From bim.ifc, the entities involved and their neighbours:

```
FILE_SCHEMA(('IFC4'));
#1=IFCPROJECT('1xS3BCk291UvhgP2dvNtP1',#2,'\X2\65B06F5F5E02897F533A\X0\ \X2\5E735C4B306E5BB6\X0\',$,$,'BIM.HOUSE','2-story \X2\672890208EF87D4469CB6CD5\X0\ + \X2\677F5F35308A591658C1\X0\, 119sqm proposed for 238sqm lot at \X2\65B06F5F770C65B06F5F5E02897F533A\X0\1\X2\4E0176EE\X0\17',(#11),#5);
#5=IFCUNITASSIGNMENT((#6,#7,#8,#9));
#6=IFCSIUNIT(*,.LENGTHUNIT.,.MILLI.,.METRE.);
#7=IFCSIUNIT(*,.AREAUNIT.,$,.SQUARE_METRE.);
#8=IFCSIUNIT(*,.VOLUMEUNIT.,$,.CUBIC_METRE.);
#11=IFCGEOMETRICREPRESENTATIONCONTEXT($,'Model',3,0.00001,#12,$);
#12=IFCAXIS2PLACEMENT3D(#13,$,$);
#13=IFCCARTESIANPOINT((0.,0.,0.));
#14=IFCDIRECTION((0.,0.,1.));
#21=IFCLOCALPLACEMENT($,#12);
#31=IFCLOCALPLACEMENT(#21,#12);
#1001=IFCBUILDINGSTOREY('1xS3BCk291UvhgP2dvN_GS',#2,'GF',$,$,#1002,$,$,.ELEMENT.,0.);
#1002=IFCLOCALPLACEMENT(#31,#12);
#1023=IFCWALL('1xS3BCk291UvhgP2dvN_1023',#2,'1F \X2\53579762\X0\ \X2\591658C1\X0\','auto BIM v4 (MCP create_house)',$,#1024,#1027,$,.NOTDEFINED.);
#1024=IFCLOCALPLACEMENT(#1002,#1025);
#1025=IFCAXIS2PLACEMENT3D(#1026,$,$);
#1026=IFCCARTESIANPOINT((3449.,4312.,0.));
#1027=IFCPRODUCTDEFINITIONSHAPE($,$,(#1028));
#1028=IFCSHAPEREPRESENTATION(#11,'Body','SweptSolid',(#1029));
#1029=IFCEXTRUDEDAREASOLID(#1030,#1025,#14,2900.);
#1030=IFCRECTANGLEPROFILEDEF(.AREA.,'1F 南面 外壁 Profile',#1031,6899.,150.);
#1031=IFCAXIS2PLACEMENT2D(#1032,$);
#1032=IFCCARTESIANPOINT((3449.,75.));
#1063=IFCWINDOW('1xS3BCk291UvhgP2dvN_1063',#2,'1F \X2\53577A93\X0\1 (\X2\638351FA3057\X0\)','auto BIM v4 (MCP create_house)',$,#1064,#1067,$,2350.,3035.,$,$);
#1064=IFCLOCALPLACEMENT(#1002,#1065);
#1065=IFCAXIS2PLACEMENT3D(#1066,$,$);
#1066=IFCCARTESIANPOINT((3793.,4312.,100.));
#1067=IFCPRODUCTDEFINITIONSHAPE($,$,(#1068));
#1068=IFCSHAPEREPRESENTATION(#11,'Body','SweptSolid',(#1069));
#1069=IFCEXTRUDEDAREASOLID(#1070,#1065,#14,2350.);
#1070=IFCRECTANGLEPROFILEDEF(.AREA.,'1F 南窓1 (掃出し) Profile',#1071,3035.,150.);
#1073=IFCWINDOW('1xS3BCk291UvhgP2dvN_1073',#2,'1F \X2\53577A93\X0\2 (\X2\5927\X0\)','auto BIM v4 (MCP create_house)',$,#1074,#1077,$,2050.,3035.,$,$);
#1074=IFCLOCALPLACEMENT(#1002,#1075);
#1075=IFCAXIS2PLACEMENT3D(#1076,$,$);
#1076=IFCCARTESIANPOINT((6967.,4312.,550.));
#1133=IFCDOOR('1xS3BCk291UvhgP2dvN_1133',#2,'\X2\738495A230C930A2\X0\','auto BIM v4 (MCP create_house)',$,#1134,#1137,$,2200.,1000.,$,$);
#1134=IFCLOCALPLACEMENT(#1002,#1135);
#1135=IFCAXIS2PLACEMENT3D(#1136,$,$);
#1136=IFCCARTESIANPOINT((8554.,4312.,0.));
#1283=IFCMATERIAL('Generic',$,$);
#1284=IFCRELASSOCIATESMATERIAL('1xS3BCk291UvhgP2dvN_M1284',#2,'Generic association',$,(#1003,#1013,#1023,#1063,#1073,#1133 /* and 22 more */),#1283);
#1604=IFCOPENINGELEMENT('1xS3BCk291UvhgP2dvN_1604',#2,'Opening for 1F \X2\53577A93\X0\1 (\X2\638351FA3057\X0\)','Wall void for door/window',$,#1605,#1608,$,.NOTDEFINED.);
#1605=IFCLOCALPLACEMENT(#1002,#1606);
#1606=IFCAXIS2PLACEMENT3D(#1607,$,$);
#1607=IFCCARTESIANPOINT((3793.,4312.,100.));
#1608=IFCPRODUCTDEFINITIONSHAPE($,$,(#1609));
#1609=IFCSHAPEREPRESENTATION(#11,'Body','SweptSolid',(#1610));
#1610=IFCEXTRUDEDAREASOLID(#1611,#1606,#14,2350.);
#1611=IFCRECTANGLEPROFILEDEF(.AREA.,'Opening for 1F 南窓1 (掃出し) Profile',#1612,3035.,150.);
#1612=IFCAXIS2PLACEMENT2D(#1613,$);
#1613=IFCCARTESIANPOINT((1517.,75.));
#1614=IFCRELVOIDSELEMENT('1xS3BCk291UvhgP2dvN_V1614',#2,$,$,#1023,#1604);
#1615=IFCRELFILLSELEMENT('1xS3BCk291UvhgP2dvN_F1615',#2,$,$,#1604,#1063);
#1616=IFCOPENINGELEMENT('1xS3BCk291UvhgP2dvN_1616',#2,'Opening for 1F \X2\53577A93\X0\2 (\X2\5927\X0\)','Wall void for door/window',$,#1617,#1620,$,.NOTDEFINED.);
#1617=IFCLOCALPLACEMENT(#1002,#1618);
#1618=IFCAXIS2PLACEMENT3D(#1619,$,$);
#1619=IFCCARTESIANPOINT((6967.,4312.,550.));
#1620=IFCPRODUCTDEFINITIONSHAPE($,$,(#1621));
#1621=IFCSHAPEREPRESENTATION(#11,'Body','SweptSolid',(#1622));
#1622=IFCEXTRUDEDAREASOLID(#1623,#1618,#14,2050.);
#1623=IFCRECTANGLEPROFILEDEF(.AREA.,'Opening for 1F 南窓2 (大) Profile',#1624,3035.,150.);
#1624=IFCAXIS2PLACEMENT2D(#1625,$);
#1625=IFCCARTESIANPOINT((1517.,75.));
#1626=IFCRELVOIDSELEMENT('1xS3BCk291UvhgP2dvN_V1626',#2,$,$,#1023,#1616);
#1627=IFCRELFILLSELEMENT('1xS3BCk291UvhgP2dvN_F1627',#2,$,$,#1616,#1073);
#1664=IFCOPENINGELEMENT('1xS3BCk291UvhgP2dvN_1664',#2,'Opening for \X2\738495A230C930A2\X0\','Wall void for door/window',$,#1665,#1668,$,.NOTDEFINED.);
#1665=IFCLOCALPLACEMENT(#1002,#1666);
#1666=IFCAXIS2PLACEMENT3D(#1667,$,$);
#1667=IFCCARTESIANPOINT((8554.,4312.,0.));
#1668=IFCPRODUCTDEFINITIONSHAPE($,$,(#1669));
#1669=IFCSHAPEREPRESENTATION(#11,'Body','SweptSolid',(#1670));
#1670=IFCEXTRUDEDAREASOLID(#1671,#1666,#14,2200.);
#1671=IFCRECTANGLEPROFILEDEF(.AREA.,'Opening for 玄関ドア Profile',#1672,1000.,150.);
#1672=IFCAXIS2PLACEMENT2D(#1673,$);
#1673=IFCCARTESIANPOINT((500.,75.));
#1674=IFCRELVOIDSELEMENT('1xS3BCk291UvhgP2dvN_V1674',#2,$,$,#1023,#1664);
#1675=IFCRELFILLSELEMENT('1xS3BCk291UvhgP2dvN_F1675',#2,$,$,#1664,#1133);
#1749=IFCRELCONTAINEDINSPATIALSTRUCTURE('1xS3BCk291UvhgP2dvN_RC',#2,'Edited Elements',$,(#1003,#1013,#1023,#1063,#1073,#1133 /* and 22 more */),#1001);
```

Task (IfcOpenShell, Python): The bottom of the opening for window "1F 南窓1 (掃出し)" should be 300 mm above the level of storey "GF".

```python
import numpy as np
import ifcopenshell
import ifcopenshell.api.geometry
import ifcopenshell.geom
import ifcopenshell.util.element
import ifcopenshell.util.placement
import ifcopenshell.util.shape
import ifcopenshell.util.unit

model = ifcopenshell.open("bim.ifc")
unit_scale = ifcopenshell.util.unit.calculate_unit_scale(model)

window = model.by_id(1063)
opening = window.FillsVoids[0].RelatingOpeningElement
storey = ifcopenshell.util.element.get_container(window, ifc_class="IfcBuildingStorey")
level = ifcopenshell.util.placement.get_local_placement(storey.ObjectPlacement)[2, 3]

# The opening's origin need not be at the sill, so measure its lowest point.
shape = ifcopenshell.geom.create_shape(ifcopenshell.geom.settings(), opening)
bottom = ifcopenshell.util.shape.get_shape_bottom_elevation(shape, shape.geometry) / unit_scale
dz = level + 300.0 - bottom

shift = np.array([0.0, 0.0, dz])
# The window is not placed relative to its opening, so move both.
for product in (opening, window):
    matrix = ifcopenshell.util.placement.get_local_placement(product.ObjectPlacement)
    matrix[:3, 3] += shift
    ifcopenshell.api.geometry.edit_object_placement(model, product=product, matrix=matrix, is_si=False)

print(f"moved by {dz * unit_scale:+.3f} m")

model.write("bim_updated.ifc")
```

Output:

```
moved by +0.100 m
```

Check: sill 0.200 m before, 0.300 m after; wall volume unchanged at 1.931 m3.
